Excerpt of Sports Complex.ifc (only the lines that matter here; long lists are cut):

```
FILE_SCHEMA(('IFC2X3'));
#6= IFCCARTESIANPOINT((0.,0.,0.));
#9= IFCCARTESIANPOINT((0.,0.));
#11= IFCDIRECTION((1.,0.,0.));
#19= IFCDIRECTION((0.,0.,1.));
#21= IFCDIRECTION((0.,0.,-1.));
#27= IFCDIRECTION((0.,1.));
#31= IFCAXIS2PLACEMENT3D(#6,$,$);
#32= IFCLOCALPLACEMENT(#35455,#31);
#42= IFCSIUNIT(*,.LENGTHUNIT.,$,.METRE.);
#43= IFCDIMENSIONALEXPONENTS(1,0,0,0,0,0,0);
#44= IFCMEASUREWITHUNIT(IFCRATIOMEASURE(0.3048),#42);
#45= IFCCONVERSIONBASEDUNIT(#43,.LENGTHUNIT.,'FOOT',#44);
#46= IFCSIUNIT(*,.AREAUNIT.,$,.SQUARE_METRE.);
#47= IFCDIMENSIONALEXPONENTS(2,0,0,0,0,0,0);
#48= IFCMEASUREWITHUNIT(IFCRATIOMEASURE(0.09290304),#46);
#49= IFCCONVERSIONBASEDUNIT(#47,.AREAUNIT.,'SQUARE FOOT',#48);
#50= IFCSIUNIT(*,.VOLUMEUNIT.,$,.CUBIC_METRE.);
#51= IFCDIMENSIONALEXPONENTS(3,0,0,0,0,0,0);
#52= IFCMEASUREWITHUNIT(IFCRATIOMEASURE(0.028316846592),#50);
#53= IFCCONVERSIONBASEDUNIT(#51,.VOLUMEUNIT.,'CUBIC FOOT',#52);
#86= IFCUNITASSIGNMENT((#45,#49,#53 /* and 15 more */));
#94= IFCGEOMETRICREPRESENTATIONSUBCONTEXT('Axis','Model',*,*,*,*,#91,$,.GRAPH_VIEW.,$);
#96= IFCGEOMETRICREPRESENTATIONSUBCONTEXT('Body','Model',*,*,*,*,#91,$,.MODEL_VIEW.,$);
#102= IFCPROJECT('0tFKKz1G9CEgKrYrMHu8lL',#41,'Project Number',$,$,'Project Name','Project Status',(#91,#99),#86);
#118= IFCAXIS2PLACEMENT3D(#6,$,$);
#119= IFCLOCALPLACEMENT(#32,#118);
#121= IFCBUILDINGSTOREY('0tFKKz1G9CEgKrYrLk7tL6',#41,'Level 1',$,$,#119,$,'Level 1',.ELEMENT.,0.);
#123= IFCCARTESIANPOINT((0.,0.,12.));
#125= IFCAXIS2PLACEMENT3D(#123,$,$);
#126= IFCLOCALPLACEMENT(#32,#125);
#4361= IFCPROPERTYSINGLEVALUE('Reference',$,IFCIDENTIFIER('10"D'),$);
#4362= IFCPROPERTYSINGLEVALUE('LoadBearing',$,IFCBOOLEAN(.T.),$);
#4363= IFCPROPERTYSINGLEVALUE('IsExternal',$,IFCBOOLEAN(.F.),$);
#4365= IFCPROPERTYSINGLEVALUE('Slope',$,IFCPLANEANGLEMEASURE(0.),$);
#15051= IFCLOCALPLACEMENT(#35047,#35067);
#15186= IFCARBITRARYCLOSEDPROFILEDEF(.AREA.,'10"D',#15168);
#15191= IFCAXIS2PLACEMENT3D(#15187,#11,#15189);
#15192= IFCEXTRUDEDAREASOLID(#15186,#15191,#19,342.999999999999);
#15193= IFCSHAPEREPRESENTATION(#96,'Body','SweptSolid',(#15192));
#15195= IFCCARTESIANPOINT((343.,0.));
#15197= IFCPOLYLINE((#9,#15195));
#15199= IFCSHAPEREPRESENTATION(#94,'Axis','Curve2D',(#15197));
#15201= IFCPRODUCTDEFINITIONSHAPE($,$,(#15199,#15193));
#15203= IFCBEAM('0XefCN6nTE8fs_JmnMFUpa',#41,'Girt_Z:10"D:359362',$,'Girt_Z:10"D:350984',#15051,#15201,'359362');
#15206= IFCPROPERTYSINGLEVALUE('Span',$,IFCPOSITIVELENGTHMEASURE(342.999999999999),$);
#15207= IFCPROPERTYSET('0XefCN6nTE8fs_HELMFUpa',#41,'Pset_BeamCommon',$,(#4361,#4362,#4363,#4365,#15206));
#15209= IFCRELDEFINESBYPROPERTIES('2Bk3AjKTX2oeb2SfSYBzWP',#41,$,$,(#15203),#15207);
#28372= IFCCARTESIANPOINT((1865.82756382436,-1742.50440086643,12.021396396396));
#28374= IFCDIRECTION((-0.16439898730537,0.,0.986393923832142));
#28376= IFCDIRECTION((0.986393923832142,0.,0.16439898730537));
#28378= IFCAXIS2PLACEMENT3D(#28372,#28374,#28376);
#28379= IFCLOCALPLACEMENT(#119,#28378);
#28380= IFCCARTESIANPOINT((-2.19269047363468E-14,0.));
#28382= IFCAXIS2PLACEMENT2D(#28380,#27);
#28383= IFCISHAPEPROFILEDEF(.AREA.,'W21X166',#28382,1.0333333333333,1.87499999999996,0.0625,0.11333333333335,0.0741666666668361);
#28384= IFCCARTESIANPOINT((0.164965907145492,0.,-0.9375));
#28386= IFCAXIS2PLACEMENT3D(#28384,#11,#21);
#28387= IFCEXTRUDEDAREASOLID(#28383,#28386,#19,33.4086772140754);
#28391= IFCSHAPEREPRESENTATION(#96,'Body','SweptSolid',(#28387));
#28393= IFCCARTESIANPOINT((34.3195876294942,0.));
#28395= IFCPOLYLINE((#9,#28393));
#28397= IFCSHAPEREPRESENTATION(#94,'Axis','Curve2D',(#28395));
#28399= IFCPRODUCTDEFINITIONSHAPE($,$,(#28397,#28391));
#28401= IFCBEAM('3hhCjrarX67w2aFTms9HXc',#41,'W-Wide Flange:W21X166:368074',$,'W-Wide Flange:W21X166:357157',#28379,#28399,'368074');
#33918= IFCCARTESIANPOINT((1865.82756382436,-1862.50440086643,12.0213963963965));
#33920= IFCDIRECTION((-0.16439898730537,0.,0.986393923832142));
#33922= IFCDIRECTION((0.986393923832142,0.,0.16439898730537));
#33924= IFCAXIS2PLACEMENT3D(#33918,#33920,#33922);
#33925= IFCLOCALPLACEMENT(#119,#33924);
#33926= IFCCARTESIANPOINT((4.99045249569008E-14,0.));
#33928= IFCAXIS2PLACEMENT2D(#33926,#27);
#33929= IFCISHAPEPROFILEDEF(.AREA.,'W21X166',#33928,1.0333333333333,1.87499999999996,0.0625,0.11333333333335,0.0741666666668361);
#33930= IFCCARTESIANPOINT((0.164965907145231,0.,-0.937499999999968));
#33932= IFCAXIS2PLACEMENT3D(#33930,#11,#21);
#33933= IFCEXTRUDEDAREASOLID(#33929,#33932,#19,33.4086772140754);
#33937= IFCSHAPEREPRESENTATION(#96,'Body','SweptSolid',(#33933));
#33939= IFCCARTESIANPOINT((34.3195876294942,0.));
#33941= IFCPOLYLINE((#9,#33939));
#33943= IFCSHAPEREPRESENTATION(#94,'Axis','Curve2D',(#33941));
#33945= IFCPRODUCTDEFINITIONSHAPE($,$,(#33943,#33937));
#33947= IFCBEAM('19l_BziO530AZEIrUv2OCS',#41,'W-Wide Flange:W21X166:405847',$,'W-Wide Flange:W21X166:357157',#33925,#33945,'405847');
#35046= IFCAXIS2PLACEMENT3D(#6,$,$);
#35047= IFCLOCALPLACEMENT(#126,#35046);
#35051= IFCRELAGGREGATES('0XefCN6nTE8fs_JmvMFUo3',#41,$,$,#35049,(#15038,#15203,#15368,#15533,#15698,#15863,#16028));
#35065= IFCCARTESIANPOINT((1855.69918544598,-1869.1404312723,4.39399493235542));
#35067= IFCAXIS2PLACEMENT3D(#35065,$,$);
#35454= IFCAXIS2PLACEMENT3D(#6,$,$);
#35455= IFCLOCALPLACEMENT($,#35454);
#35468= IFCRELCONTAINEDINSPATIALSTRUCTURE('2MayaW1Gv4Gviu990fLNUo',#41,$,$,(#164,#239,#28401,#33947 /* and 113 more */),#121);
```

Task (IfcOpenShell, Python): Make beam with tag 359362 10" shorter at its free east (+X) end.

```python
import numpy as np
import ifcopenshell
import ifcopenshell.api.pset
import ifcopenshell.util.element
import ifcopenshell.util.representation
import ifcopenshell.util.unit

model = ifcopenshell.open("Sports Complex.ifc")
unit_scale = ifcopenshell.util.unit.calculate_unit_scale(model)

member = model.by_id(15203)
change = -10 * 0.0254 / unit_scale

# The extrusion runs towards the end named, so only its depth changes.
body = ifcopenshell.util.representation.get_representation(member, "Model", "Body")
solid = body.Items[0]
old_length = solid.Depth
solid.Depth += change

# Move the axis end point with it.
axis = next(r for r in member.Representation.Representations if r.RepresentationIdentifier == "Axis").Items[0]
start, end = (np.array(p.Coordinates) for p in axis.Points)
end = end + (end - start) / np.linalg.norm(end - start) * change
point = model.createIfcCartesianPoint(end.tolist())
axis.Points = [axis.Points[0], point]

# Update the stored length and volume.
pset = model.by_id(ifcopenshell.util.element.get_pset(member, "Pset_BeamCommon", should_inherit=False)["id"])
ifcopenshell.api.pset.edit_pset(model, pset=pset, properties={
    "Span": model.create_entity("IfcPositiveLengthMeasure", solid.Depth),
})

print(f"length {old_length:g} -> {solid.Depth:g}")

model.write("Sports Complex-out.ifc")
```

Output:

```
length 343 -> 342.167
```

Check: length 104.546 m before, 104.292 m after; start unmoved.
